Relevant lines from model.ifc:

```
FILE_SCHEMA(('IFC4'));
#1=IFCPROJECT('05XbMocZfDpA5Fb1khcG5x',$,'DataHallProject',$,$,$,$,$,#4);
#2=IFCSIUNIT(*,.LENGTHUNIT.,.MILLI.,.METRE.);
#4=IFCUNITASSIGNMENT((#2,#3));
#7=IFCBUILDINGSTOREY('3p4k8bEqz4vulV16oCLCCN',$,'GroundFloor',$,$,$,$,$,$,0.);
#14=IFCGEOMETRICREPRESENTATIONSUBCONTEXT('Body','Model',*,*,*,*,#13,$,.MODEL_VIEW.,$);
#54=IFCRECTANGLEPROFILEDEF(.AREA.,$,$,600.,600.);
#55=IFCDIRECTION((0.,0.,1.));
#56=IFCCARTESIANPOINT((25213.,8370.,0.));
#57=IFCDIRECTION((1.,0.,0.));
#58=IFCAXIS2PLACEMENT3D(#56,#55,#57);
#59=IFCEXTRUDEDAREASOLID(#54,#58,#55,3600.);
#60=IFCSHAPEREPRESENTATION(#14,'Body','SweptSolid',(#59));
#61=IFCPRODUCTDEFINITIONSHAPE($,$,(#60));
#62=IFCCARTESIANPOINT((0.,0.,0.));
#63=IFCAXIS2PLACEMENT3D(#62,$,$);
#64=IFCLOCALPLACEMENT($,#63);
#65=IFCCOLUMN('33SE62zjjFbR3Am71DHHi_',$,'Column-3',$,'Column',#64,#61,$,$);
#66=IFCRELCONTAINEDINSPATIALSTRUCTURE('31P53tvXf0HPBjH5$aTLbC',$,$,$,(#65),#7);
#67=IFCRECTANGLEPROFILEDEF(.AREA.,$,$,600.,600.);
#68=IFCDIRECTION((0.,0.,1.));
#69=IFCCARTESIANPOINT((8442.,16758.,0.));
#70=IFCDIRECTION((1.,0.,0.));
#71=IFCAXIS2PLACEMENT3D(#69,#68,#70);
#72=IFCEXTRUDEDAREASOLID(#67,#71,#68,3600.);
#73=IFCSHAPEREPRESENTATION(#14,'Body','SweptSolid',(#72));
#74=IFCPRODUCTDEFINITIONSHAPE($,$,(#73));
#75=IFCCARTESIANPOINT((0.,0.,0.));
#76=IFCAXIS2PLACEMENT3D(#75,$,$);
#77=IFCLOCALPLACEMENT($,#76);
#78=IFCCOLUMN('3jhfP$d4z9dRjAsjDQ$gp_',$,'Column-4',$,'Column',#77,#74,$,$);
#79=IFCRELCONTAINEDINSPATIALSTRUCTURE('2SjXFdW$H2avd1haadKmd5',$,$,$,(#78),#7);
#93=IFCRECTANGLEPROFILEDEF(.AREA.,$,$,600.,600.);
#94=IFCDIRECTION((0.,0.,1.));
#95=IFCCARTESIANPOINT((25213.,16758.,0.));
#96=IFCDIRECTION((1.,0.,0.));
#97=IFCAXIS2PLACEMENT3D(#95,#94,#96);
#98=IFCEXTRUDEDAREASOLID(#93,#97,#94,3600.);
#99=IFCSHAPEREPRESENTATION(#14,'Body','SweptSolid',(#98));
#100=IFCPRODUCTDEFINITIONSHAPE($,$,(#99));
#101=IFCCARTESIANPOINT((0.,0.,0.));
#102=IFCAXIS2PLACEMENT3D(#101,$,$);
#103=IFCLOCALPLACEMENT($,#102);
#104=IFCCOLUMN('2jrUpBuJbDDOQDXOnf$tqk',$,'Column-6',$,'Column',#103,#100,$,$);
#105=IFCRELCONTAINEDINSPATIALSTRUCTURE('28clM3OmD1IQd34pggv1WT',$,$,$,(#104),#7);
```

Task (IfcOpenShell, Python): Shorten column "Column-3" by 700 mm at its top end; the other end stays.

```python
import ifcopenshell
import ifcopenshell.util.representation
import ifcopenshell.util.unit

model = ifcopenshell.open("model.ifc")
unit_scale = ifcopenshell.util.unit.calculate_unit_scale(model)

member = model.by_guid("33SE62zjjFbR3Am71DHHi_")
change = -0.7 / unit_scale

# The extrusion runs towards the end named, so only its depth changes.
body = ifcopenshell.util.representation.get_representation(member, "Model", "Body")
solid = body.Items[0]
old_length = solid.Depth
solid.Depth += change

print(f"length {old_length:g} -> {solid.Depth:g}")

model.write("model_rev.ifc")
```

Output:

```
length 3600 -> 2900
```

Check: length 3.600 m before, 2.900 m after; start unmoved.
